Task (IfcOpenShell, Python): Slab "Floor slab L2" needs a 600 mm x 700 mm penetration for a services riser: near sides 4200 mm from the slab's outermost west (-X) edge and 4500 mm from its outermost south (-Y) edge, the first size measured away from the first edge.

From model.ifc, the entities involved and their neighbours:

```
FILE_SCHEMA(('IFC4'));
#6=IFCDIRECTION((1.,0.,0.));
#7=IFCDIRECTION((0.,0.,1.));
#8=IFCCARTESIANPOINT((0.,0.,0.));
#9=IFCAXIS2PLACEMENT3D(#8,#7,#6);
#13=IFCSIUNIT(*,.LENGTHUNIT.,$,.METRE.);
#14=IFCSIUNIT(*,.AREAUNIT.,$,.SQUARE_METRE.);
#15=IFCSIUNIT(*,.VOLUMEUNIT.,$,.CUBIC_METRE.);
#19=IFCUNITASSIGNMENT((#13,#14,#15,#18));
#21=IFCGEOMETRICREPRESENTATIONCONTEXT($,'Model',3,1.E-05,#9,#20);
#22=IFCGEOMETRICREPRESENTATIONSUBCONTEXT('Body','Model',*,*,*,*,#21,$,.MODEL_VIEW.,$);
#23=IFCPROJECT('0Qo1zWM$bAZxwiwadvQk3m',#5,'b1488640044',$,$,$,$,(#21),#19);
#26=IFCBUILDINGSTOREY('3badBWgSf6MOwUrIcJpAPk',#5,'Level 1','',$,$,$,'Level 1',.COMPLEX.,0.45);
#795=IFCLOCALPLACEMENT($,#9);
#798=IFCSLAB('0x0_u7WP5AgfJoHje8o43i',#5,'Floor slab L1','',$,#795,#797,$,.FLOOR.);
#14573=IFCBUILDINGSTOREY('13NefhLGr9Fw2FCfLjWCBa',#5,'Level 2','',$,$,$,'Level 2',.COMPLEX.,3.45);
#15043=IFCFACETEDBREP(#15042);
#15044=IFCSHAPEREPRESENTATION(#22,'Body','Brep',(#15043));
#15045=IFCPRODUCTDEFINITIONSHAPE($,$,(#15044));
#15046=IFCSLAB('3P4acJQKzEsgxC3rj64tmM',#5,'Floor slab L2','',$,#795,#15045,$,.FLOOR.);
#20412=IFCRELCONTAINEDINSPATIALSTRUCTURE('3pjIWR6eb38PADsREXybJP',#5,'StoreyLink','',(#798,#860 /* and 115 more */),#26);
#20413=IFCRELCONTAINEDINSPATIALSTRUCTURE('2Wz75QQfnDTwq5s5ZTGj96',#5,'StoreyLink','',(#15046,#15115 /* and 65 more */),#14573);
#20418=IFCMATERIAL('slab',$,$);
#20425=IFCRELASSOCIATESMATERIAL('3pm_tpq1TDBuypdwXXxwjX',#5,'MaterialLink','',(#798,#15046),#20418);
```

```python
import numpy as np
import ifcopenshell
import ifcopenshell.api.feature
import ifcopenshell.api.geometry
import ifcopenshell.api.root
import ifcopenshell.geom
import ifcopenshell.util.placement
import ifcopenshell.util.representation
import ifcopenshell.util.shape
import ifcopenshell.util.unit

model = ifcopenshell.open("model.ifc")
unit_scale = ifcopenshell.util.unit.calculate_unit_scale(model)
settings = ifcopenshell.geom.settings()


def volume(element):
    """Net volume in cubic metres, openings subtracted."""
    shape = ifcopenshell.geom.create_shape(settings, element)
    return ifcopenshell.util.shape.get_volume(shape.geometry)


slab = model.by_guid("3P4acJQKzEsgxC3rj64tmM")
before = volume(slab)

# Extent in the slab's own axes, in metres. The edges named are its -X and -Y sides.
slab_shape = ifcopenshell.geom.create_shape(settings, slab)
vertices = ifcopenshell.util.shape.get_vertices(slab_shape.geometry)
x_min, y_min, bottom = vertices.min(axis=0)
top = vertices[:, 2].max()

opening = ifcopenshell.api.root.create_entity(model, ifc_class="IfcOpeningElement", name="Services riser opening", predefined_type="OPENING")
context = ifcopenshell.util.representation.get_context(model, "Model", "Body", "MODEL_VIEW")
width, depth = 0.6, 0.7
outline = [(0.0, 0.0), (width, 0.0), (width, depth), (0.0, depth), (0.0, 0.0)]
# Overshoot both faces by 50 mm so the cut is clean.
shape = ifcopenshell.api.geometry.add_slab_representation(
    model, context=context, depth=top - bottom + 0.1, polyline=outline
)
ifcopenshell.api.geometry.assign_representation(model, product=opening, representation=shape)

matrix = ifcopenshell.util.placement.get_local_placement(slab.ObjectPlacement)
matrix[:, 3] = matrix @ np.append(np.array([x_min + 4.2, y_min + 4.5, bottom - 0.05]) / unit_scale, 1.0)
ifcopenshell.api.geometry.edit_object_placement(model, product=opening, matrix=matrix, is_si=False)
ifcopenshell.api.feature.add_feature(model, feature=opening, element=slab)

after = volume(slab)

print(f"slab volume {before:.3f} -> {after:.3f} m3")

model.write("model_rev.ifc")
```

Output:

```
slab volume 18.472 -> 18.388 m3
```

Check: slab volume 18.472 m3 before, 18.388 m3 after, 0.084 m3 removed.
